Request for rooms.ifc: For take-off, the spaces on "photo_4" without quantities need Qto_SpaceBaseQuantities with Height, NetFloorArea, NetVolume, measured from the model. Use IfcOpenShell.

First a look at what the model holds.

```python
import ifcopenshell
import ifcopenshell.util.element
import ifcopenshell.util.unit

model = ifcopenshell.open("rooms.ifc")
print(model.schema)
for unit_type in ("LENGTHUNIT", "AREAUNIT", "VOLUMEUNIT"):
    print(unit_type, ifcopenshell.util.unit.calculate_unit_scale(model, unit_type))
storey = next(s for s in model.by_type("IfcBuildingStorey") if s.Name == "photo_4")
spaces = [e for e in ifcopenshell.util.element.get_decomposition(storey) if e.is_a("IfcSpace")]
for e in sorted(spaces, key=lambda e: e.id()):
    print(e.id(), e.is_a(), e.Name, list(ifcopenshell.util.element.get_psets(e, qtos_only=True)), sep=" | ")
```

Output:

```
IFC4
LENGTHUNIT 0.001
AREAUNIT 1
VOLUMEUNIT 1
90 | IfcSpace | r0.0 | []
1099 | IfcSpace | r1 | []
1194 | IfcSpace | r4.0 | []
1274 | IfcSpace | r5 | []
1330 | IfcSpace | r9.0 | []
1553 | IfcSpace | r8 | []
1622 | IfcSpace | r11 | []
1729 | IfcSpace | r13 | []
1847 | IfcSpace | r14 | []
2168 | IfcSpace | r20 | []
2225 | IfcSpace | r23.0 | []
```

```python
import ifcopenshell
import ifcopenshell.api.pset
import ifcopenshell.geom
import ifcopenshell.util.element
import ifcopenshell.util.shape
import ifcopenshell.util.unit

model = ifcopenshell.open("rooms.ifc")
unit_scale = ifcopenshell.util.unit.calculate_unit_scale(model)
area_scale = ifcopenshell.util.unit.calculate_unit_scale(model, "AREAUNIT")
volume_scale = ifcopenshell.util.unit.calculate_unit_scale(model, "VOLUMEUNIT")
settings = ifcopenshell.geom.settings()

storey = next(s for s in model.by_type("IfcBuildingStorey") if s.Name == "photo_4")
spaces = [e for e in ifcopenshell.util.element.get_decomposition(storey) if e.is_a("IfcSpace")]

for e in sorted(spaces, key=lambda e: e.id()):
    if ifcopenshell.util.element.get_psets(e, qtos_only=True, should_inherit=False):
        continue
    # Geometry comes back in metres, in the element's own axes.
    shape = ifcopenshell.geom.create_shape(settings, e)
    values = {
        "Height": ifcopenshell.util.shape.get_z(shape.geometry) / unit_scale,
        "NetFloorArea": ifcopenshell.util.shape.get_footprint_area(shape.geometry) / area_scale,
        "NetVolume": ifcopenshell.util.shape.get_volume(shape.geometry) / volume_scale,
    }
    qto = ifcopenshell.api.pset.add_qto(model, product=e, name="Qto_SpaceBaseQuantities")
    ifcopenshell.api.pset.edit_qto(model, qto=qto, properties=values)
    print(e.id(), {k: round(v, 3) for k, v in values.items()})

model.write("rooms_v2.ifc")
```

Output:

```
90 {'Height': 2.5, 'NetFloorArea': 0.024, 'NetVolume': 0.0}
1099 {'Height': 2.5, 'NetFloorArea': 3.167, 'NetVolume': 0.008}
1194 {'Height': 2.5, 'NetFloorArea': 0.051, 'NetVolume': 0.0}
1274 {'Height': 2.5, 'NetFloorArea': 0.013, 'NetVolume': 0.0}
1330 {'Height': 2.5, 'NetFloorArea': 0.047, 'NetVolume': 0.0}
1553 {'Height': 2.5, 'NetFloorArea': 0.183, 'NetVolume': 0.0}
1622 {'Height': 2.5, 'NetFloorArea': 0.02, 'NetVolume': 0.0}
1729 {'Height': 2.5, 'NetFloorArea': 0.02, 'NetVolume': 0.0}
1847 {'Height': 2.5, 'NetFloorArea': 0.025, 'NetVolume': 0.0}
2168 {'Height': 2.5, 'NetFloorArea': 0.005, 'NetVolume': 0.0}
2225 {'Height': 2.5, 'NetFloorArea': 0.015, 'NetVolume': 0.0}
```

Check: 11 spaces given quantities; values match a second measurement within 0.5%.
